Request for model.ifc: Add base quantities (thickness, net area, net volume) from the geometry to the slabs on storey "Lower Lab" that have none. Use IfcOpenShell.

First a look at what the model holds.

```python
import ifcopenshell
import ifcopenshell.util.element
import ifcopenshell.util.unit

model = ifcopenshell.open("model.ifc")
print(model.schema)
for unit_type in ("LENGTHUNIT", "AREAUNIT", "VOLUMEUNIT"):
    print(unit_type, ifcopenshell.util.unit.calculate_unit_scale(model, unit_type))
storey = next(s for s in model.by_type("IfcBuildingStorey") if s.Name == "Lower Lab")
slabs = [e for e in ifcopenshell.util.element.get_decomposition(storey) if e.is_a("IfcSlab")]
for e in sorted(slabs, key=lambda e: e.id()):
    print(e.id(), e.is_a(), e.Name, list(ifcopenshell.util.element.get_psets(e, qtos_only=True)), sep=" | ")
```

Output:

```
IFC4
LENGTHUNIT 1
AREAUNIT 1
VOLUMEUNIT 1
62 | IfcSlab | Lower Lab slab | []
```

```python
import ifcopenshell
import ifcopenshell.api.pset
import ifcopenshell.geom
import ifcopenshell.util.element
import ifcopenshell.util.shape
import ifcopenshell.util.unit

model = ifcopenshell.open("model.ifc")
unit_scale = ifcopenshell.util.unit.calculate_unit_scale(model)
area_scale = ifcopenshell.util.unit.calculate_unit_scale(model, "AREAUNIT")
volume_scale = ifcopenshell.util.unit.calculate_unit_scale(model, "VOLUMEUNIT")
settings = ifcopenshell.geom.settings()

storey = next(s for s in model.by_type("IfcBuildingStorey") if s.Name == "Lower Lab")
slabs = [e for e in ifcopenshell.util.element.get_decomposition(storey) if e.is_a("IfcSlab")]

for e in sorted(slabs, key=lambda e: e.id()):
    if ifcopenshell.util.element.get_psets(e, qtos_only=True, should_inherit=False):
        continue
    # Geometry comes back in metres, in the element's own axes.
    shape = ifcopenshell.geom.create_shape(settings, e)
    values = {
        "Width": ifcopenshell.util.shape.get_z(shape.geometry) / unit_scale,
        "NetArea": ifcopenshell.util.shape.get_footprint_area(shape.geometry) / area_scale,
        "NetVolume": ifcopenshell.util.shape.get_volume(shape.geometry) / volume_scale,
    }
    qto = ifcopenshell.api.pset.add_qto(model, product=e, name="Qto_SlabBaseQuantities")
    ifcopenshell.api.pset.edit_qto(model, qto=qto, properties=values)
    print(e.id(), {k: round(v, 3) for k, v in values.items()})

model.write("model_rev.ifc")
```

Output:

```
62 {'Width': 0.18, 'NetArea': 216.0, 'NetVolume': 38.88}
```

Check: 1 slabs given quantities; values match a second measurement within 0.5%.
